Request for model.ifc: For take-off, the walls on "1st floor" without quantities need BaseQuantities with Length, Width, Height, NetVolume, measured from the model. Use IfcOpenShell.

First a look at what the model holds.

```python
import ifcopenshell
import ifcopenshell.util.element
import ifcopenshell.util.unit

model = ifcopenshell.open("model.ifc")
print(model.schema)
for unit_type in ("LENGTHUNIT", "AREAUNIT", "VOLUMEUNIT"):
    print(unit_type, ifcopenshell.util.unit.calculate_unit_scale(model, unit_type))
storey = next(s for s in model.by_type("IfcBuildingStorey") if s.Name == "1st floor")
walls = [e for e in ifcopenshell.util.element.get_decomposition(storey) if e.is_a("IfcWall")]
for e in sorted(walls, key=lambda e: e.id()):
    print(e.id(), e.is_a(), e.Name, list(ifcopenshell.util.element.get_psets(e, qtos_only=True)), sep=" | ")
```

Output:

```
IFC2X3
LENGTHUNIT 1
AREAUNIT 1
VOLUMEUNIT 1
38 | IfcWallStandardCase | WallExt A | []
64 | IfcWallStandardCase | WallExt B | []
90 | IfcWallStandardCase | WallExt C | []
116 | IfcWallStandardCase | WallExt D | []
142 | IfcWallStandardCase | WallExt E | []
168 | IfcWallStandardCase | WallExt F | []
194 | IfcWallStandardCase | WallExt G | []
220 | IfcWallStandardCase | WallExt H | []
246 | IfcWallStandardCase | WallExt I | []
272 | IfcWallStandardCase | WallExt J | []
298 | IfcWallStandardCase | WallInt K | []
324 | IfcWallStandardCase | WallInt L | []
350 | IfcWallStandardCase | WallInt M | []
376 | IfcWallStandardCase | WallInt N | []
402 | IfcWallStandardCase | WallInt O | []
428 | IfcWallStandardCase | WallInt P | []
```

```python
import ifcopenshell
import ifcopenshell.api.pset
import ifcopenshell.geom
import ifcopenshell.util.element
import ifcopenshell.util.shape
import ifcopenshell.util.unit

model = ifcopenshell.open("model.ifc")
unit_scale = ifcopenshell.util.unit.calculate_unit_scale(model)
volume_scale = ifcopenshell.util.unit.calculate_unit_scale(model, "VOLUMEUNIT")
settings = ifcopenshell.geom.settings()

storey = next(s for s in model.by_type("IfcBuildingStorey") if s.Name == "1st floor")
walls = [e for e in ifcopenshell.util.element.get_decomposition(storey) if e.is_a("IfcWall")]

for e in sorted(walls, key=lambda e: e.id()):
    if ifcopenshell.util.element.get_psets(e, qtos_only=True, should_inherit=False):
        continue
    # Geometry comes back in metres, in the element's own axes.
    shape = ifcopenshell.geom.create_shape(settings, e)
    values = {
        "Length": ifcopenshell.util.shape.get_x(shape.geometry) / unit_scale,
        "Width": ifcopenshell.util.shape.get_y(shape.geometry) / unit_scale,
        "Height": ifcopenshell.util.shape.get_z(shape.geometry) / unit_scale,
        "NetVolume": ifcopenshell.util.shape.get_volume(shape.geometry) / volume_scale,
    }
    qto = ifcopenshell.api.pset.add_qto(model, product=e, name="BaseQuantities")
    ifcopenshell.api.pset.edit_qto(model, qto=qto, properties=values)
    print(e.id(), {k: round(v, 3) for k, v in values.items()})

model.write("model_rev.ifc")
```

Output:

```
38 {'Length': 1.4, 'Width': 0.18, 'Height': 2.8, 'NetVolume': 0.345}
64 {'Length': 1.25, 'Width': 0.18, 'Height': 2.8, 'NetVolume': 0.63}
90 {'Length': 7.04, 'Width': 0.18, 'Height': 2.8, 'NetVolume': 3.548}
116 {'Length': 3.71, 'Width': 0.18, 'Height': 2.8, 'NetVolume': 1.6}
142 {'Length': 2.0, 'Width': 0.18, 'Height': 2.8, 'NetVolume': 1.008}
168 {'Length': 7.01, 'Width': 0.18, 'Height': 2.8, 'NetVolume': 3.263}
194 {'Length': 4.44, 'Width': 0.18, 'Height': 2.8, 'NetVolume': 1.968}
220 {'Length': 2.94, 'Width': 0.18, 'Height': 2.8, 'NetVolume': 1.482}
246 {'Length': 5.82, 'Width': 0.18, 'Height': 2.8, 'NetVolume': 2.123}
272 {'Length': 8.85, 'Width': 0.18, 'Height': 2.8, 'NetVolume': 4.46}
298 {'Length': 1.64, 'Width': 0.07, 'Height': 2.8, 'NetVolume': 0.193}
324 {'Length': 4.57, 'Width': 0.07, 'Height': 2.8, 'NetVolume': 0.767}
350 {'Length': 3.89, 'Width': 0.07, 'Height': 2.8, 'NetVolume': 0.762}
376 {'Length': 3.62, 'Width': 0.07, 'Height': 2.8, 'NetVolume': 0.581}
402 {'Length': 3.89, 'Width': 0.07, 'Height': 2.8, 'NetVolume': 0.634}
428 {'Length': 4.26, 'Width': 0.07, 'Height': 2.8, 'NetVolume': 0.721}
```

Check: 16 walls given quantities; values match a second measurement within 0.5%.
